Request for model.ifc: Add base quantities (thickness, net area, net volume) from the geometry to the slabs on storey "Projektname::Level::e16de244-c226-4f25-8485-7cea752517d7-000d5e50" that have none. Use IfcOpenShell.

First a look at what the model holds.

```python
import ifcopenshell
import ifcopenshell.util.element
import ifcopenshell.util.unit

model = ifcopenshell.open("model.ifc")
print(model.schema)
for unit_type in ("LENGTHUNIT", "AREAUNIT", "VOLUMEUNIT"):
    print(unit_type, ifcopenshell.util.unit.calculate_unit_scale(model, unit_type))
storey = next(s for s in model.by_type("IfcBuildingStorey") if s.Name == "Projektname::Level::e16de244-c226-4f25-8485-7cea752517d7-000d5e50")
slabs = [e for e in ifcopenshell.util.element.get_decomposition(storey) if e.is_a("IfcSlab")]
for e in sorted(slabs, key=lambda e: e.id()):
    print(e.id(), e.is_a(), e.Name, list(ifcopenshell.util.element.get_psets(e, qtos_only=True)), sep=" | ")
```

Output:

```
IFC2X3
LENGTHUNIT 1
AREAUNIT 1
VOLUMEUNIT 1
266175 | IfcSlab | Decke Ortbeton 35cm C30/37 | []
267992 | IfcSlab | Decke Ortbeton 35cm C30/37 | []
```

```python
import ifcopenshell
import ifcopenshell.api.pset
import ifcopenshell.geom
import ifcopenshell.util.element
import ifcopenshell.util.shape
import ifcopenshell.util.unit

model = ifcopenshell.open("model.ifc")
unit_scale = ifcopenshell.util.unit.calculate_unit_scale(model)
area_scale = ifcopenshell.util.unit.calculate_unit_scale(model, "AREAUNIT")
volume_scale = ifcopenshell.util.unit.calculate_unit_scale(model, "VOLUMEUNIT")
settings = ifcopenshell.geom.settings()

storey = next(s for s in model.by_type("IfcBuildingStorey") if s.Name == "Projektname::Level::e16de244-c226-4f25-8485-7cea752517d7-000d5e50")
slabs = [e for e in ifcopenshell.util.element.get_decomposition(storey) if e.is_a("IfcSlab")]

for e in sorted(slabs, key=lambda e: e.id()):
    if ifcopenshell.util.element.get_psets(e, qtos_only=True, should_inherit=False):
        continue
    # Geometry comes back in metres, in the element's own axes.
    shape = ifcopenshell.geom.create_shape(settings, e)
    values = {
        "Width": ifcopenshell.util.shape.get_z(shape.geometry) / unit_scale,
        "NetArea": ifcopenshell.util.shape.get_footprint_area(shape.geometry) / area_scale,
        "NetVolume": ifcopenshell.util.shape.get_volume(shape.geometry) / volume_scale,
    }
    qto = ifcopenshell.api.pset.add_qto(model, product=e, name="BaseQuantities")
    ifcopenshell.api.pset.edit_qto(model, qto=qto, properties=values)
    print(e.id(), {k: round(v, 3) for k, v in values.items()})

model.write("model_v2.ifc")
```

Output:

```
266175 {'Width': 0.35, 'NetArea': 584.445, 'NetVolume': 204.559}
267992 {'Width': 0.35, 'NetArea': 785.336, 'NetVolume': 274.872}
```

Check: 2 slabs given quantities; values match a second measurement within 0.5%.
